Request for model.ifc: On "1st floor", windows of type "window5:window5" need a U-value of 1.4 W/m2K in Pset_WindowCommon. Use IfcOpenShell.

First a look at what the model holds.

```python
import ifcopenshell
import ifcopenshell.util.element

model = ifcopenshell.open("model.ifc")
print(model.schema)
storey = next(s for s in model.by_type("IfcBuildingStorey") if s.Name == "1st floor")
windows = [e for e in ifcopenshell.util.element.get_decomposition(storey) if e.is_a("IfcWindow")]
seen = {}
for e in windows:
    element_type = ifcopenshell.util.element.get_type(e)
    key = (element_type.Name if element_type != e and element_type else None, ifcopenshell.util.element.get_pset(e, "Pset_WindowCommon", "ThermalTransmittance"))
    seen[key] = seen.get(key, 0) + 1
for (name, value), count in sorted(seen.items(), key=str):
    print(count, "x", name, "|", value)
```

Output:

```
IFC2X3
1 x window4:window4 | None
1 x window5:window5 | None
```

```python
import ifcopenshell
import ifcopenshell.api.pset
import ifcopenshell.util.element

model = ifcopenshell.open("model.ifc")

storey = next(s for s in model.by_type("IfcBuildingStorey") if s.Name == "1st floor")
windows = [e for e in ifcopenshell.util.element.get_decomposition(storey) if e.is_a("IfcWindow")]

count = 0
for e in windows:
    element_type = ifcopenshell.util.element.get_type(e)
    if element_type in (None, e) or element_type.Name != "window5:window5":
        continue
    # add_pset returns the element's existing set when there is one.
    pset = ifcopenshell.api.pset.add_pset(model, product=e, name="Pset_WindowCommon")
    ifcopenshell.api.pset.edit_pset(model, pset=pset, properties={"ThermalTransmittance": 1.4})
    count += 1

print(count, "windows updated")

model.write("model-out.ifc")
```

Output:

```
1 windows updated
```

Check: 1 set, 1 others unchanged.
